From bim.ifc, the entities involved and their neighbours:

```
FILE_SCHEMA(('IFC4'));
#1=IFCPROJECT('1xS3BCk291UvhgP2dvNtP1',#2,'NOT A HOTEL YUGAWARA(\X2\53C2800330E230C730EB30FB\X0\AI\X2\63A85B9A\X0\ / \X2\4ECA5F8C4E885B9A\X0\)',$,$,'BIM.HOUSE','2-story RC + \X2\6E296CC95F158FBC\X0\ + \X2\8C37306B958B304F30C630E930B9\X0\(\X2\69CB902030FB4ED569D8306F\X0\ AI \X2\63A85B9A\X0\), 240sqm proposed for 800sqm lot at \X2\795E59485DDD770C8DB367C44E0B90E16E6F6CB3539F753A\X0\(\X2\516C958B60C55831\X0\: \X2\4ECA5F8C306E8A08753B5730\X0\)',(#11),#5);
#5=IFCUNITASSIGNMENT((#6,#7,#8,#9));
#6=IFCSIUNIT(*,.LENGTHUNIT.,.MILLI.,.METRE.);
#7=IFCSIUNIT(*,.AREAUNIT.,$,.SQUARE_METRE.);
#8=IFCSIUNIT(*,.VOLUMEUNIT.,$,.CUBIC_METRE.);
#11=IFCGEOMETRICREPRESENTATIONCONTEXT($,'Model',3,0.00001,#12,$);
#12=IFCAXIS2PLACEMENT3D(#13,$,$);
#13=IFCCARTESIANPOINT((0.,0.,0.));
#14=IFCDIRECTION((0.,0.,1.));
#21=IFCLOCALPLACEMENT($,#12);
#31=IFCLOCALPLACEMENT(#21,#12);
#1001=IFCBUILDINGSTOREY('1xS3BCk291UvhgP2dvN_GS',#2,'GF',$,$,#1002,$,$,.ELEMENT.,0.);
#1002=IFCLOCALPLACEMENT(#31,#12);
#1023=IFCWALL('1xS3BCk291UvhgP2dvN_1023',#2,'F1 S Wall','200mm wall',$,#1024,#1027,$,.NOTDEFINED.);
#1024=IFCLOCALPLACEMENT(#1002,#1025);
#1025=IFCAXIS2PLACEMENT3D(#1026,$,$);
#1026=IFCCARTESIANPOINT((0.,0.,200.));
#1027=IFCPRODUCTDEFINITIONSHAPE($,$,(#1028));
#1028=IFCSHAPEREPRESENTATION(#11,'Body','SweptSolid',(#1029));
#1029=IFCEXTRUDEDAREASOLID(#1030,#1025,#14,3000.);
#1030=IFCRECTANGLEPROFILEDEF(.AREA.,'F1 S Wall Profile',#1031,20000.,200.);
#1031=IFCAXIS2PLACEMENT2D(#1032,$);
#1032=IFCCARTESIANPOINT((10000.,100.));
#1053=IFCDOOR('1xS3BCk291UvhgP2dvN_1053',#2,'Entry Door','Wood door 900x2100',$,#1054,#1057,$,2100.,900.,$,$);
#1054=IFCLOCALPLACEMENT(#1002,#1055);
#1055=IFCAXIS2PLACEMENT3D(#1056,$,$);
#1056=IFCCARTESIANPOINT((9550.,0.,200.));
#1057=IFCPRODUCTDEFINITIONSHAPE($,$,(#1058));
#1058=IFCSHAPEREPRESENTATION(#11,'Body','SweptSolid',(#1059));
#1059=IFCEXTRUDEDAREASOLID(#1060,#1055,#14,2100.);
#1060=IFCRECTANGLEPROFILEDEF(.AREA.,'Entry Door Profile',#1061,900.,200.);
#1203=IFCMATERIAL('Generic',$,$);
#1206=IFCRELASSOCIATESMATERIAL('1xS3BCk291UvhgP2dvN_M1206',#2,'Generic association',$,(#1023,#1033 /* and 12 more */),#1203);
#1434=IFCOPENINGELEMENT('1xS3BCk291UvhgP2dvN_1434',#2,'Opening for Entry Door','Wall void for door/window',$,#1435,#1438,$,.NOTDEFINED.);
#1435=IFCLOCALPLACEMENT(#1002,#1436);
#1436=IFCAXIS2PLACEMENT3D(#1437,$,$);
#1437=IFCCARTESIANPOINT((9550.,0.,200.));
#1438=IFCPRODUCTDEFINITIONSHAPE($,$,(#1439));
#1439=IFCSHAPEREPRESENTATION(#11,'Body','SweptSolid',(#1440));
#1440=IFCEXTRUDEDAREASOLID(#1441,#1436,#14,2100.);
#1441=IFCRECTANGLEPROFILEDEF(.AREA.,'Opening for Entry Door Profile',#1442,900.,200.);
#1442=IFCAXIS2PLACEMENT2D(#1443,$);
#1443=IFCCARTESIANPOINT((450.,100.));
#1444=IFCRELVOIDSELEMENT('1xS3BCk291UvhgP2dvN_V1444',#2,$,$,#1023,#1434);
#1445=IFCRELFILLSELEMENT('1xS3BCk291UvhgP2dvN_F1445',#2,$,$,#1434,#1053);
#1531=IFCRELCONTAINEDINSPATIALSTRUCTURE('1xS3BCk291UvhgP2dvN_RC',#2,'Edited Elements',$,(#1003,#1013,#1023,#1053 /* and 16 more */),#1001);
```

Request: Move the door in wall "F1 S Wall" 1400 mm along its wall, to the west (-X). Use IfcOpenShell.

```python
import ifcopenshell
import ifcopenshell.api.geometry
import ifcopenshell.util.placement

model = ifcopenshell.open("bim.ifc")

door = model.by_guid("1xS3BCk291UvhgP2dvN_1053")
opening = door.FillsVoids[0].RelatingOpeningElement
wall = opening.VoidsElements[0].RelatingBuildingElement

wall_matrix = ifcopenshell.util.placement.get_local_placement(wall.ObjectPlacement)
shift = wall_matrix[:3, 0] * -1400.0
before = ifcopenshell.util.placement.get_local_placement(door.ObjectPlacement)[:3, 3].copy()

# The door is not placed relative to its opening, so move both.
for product in (opening, door):
    matrix = ifcopenshell.util.placement.get_local_placement(product.ObjectPlacement)
    matrix[:3, 3] += shift
    ifcopenshell.api.geometry.edit_object_placement(model, product=product, matrix=matrix, is_si=False)

after = ifcopenshell.util.placement.get_local_placement(door.ObjectPlacement)[:3, 3]
print("door moved by", (after - before).round(3) + 0.0)

model.write("bim_v2.ifc")
```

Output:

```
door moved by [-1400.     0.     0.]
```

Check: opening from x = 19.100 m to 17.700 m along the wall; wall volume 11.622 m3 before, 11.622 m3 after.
